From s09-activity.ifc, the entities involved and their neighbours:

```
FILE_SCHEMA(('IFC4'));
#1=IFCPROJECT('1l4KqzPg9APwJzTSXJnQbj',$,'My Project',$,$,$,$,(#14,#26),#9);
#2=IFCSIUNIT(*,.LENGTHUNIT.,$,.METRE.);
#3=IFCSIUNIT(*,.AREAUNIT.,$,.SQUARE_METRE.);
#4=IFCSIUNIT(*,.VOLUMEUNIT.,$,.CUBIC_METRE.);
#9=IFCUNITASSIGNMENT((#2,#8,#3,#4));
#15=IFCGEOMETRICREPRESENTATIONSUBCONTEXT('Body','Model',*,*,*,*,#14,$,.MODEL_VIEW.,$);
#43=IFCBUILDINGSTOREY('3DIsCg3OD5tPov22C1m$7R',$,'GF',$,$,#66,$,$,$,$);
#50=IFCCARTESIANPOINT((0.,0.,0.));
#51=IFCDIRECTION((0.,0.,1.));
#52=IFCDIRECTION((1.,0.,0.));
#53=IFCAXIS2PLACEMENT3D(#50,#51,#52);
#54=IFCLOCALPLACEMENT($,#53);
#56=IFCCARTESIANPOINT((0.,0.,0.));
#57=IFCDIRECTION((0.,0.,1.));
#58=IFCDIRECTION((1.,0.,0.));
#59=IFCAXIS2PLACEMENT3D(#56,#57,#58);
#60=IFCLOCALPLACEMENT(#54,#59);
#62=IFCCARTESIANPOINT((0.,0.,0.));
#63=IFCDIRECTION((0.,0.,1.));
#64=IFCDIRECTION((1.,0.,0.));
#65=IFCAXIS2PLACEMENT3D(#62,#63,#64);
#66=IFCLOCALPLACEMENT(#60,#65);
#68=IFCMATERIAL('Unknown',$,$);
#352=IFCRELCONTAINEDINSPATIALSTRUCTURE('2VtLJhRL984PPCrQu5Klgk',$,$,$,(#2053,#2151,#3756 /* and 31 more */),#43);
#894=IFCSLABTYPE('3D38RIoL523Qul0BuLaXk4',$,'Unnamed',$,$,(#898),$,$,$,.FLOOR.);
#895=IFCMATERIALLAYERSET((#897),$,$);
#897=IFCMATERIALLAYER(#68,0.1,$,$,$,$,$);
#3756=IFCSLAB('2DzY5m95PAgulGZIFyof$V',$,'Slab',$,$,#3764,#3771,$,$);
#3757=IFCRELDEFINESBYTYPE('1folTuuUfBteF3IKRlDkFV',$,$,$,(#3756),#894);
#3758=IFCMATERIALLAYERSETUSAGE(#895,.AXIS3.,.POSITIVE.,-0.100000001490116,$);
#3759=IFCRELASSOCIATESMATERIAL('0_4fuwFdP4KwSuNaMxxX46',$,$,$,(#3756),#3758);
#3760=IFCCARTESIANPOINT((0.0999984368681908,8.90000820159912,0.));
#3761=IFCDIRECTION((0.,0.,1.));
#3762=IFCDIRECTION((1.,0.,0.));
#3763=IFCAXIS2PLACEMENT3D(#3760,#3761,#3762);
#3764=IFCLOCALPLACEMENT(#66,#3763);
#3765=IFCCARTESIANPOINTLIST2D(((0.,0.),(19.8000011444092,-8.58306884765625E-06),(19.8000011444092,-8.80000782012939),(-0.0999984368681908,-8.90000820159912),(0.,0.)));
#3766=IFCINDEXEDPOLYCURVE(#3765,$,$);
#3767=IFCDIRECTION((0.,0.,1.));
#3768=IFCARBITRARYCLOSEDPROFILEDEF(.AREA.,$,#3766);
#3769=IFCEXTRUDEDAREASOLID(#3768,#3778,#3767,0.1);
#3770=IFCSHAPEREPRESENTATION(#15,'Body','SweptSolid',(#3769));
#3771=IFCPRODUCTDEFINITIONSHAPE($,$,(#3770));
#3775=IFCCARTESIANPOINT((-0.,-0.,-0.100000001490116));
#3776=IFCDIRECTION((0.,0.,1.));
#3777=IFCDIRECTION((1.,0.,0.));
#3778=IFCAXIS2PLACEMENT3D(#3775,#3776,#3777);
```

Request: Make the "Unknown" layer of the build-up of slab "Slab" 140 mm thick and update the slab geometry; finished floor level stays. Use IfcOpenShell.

```python
import ifcopenshell
import ifcopenshell.util.element
import ifcopenshell.util.representation
import ifcopenshell.util.unit

model = ifcopenshell.open("s09-activity.ifc")
unit_scale = ifcopenshell.util.unit.calculate_unit_scale(model)

layer_set = model.by_id(895)
layer = next(l for l in layer_set.MaterialLayers if l.Material and l.Material.Name == "Unknown")
change = 0.14 / unit_scale - layer.LayerThickness
layer.LayerThickness += change

# Geometry does not follow the layer set by itself.
slabs = [e for e in ifcopenshell.util.element.get_elements_by_material(model, layer_set) if e.is_a("IfcSlab")]
for slab in sorted(slabs, key=lambda e: e.id()):
    body = ifcopenshell.util.representation.get_representation(slab, "Model", "Body")
    solid = body.Items[0]
    old_depth = solid.Depth
    solid.Depth += change
    # Extruded upwards: lower the start of the extrusion so the top stays.
    x, y, z = solid.Position.Location.Coordinates
    solid.Position.Location = model.createIfcCartesianPoint((x, y, z - change))
    print(slab.id(), f"{old_depth:g} -> {solid.Depth:g}")

# The layers are counted up from the underside, which has moved.
for usage in {ifcopenshell.util.element.get_material(slab) for slab in slabs}:
    usage.OffsetFromReferenceLine -= change

model.write("s09-activity-out.ifc")
```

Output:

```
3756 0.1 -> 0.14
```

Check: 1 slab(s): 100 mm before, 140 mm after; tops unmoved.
